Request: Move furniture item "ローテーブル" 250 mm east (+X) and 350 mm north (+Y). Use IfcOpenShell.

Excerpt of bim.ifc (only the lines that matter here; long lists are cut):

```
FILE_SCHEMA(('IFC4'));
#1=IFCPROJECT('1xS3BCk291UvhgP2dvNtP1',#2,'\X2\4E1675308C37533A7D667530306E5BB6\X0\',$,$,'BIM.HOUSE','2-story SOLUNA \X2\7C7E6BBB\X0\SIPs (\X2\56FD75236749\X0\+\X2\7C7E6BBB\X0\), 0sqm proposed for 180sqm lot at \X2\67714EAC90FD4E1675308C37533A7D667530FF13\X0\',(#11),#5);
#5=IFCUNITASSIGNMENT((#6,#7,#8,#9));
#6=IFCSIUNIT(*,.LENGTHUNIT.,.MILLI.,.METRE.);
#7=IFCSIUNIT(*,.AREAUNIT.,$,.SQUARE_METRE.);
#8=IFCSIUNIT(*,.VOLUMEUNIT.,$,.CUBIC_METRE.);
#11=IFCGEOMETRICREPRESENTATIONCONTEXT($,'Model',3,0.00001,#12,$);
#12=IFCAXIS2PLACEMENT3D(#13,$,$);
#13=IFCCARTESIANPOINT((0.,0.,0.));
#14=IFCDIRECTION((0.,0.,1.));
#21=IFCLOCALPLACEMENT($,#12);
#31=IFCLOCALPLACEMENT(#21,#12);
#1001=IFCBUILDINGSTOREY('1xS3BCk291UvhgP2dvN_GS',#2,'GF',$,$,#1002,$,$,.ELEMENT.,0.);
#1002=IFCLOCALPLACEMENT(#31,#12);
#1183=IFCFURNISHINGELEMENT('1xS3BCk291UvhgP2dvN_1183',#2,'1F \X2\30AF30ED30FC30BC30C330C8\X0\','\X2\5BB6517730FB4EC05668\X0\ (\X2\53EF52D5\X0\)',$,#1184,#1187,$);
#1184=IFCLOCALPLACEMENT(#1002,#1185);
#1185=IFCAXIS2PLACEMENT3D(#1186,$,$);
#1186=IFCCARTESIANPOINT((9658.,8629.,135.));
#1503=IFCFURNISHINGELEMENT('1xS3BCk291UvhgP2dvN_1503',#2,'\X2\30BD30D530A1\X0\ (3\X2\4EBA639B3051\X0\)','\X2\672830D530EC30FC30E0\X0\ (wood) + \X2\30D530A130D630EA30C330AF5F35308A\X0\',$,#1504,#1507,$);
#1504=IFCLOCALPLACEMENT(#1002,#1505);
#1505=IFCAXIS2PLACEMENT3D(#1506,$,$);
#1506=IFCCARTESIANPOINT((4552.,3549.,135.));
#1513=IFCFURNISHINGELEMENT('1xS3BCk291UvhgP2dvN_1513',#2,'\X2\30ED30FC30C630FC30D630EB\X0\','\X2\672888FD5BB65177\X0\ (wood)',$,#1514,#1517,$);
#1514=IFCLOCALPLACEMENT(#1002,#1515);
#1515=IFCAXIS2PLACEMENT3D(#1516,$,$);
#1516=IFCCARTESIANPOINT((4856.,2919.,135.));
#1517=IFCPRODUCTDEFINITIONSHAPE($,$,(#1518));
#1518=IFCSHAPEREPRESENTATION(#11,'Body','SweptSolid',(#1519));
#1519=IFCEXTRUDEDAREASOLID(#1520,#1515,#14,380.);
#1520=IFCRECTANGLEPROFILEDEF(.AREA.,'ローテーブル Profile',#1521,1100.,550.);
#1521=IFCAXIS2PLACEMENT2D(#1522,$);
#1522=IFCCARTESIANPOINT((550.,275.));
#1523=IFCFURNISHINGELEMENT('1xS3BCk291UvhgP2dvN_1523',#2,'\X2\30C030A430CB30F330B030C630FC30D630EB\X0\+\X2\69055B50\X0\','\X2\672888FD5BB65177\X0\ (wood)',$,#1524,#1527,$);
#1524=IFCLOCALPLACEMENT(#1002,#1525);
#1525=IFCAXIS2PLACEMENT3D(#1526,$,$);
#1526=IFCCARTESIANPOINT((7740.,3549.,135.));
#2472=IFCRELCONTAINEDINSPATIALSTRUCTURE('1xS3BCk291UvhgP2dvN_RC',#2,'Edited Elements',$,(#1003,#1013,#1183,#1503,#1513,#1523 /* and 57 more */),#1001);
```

```python
import ifcopenshell
import ifcopenshell.api.geometry
import ifcopenshell.util.placement
import ifcopenshell.util.unit

model = ifcopenshell.open("bim.ifc")
unit_scale = ifcopenshell.util.unit.calculate_unit_scale(model)

item = model.by_guid("1xS3BCk291UvhgP2dvN_1513")
matrix = ifcopenshell.util.placement.get_local_placement(item.ObjectPlacement)
matrix[0, 3] += 0.25 / unit_scale
matrix[1, 3] += 0.35 / unit_scale
ifcopenshell.api.geometry.edit_object_placement(model, product=item, matrix=matrix, is_si=False)

print(ifcopenshell.util.placement.get_local_placement(item.ObjectPlacement).round(3) + 0.0)

model.write("bim_edited.ifc")
```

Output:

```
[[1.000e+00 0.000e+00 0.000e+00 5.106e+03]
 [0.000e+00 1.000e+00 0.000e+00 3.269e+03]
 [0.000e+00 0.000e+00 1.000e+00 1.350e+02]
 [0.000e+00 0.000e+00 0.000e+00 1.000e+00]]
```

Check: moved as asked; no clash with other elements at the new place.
